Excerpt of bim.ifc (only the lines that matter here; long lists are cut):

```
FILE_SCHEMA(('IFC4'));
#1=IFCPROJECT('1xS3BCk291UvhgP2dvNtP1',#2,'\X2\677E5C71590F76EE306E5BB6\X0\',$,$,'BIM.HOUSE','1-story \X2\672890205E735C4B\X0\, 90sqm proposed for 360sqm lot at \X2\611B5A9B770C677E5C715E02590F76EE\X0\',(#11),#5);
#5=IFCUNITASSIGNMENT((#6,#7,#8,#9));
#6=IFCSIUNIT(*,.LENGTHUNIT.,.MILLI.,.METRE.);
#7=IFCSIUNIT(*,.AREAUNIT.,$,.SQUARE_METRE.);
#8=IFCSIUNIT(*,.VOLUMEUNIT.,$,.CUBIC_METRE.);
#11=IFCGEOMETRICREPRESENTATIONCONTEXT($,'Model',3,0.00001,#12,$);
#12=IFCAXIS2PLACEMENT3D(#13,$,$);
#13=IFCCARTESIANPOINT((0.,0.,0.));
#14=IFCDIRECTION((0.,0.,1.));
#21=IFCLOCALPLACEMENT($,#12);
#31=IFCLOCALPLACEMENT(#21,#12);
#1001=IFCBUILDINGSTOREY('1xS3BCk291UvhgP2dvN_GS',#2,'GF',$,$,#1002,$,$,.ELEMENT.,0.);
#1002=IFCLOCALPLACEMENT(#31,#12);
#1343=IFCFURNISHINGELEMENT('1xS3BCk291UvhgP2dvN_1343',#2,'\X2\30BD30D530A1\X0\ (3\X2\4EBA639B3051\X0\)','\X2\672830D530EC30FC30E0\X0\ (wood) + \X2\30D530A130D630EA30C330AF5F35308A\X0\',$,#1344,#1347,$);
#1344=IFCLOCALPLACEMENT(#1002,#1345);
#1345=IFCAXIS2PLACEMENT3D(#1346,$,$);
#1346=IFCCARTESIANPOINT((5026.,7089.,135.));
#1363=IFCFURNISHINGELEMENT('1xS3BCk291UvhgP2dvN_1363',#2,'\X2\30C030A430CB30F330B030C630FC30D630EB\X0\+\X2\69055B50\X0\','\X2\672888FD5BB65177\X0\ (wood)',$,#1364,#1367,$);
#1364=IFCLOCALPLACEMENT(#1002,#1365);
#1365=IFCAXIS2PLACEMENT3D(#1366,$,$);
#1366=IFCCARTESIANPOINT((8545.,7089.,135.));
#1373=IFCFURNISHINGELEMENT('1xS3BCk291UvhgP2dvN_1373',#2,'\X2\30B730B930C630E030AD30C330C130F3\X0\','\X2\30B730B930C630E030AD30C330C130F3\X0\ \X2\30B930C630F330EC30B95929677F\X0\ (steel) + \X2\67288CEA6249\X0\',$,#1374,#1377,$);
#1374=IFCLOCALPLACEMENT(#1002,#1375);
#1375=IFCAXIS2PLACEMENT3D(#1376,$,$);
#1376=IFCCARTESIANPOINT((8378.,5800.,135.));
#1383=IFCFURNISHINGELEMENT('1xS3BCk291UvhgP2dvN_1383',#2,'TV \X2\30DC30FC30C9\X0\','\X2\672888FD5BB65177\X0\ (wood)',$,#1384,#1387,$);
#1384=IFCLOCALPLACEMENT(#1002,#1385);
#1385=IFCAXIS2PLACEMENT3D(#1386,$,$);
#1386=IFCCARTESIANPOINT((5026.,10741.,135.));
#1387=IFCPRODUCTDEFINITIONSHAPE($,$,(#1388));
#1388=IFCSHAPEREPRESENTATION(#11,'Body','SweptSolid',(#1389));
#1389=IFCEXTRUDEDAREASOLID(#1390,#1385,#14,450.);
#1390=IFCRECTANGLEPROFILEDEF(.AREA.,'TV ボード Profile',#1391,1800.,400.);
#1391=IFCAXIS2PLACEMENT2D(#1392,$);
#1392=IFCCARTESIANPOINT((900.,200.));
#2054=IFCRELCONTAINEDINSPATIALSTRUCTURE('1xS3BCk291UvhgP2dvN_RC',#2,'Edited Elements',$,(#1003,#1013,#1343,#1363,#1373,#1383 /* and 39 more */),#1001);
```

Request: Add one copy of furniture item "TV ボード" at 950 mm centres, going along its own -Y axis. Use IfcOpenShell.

```python
import ifcopenshell
import ifcopenshell.api.geometry
import ifcopenshell.api.root
import ifcopenshell.util.element
import ifcopenshell.util.placement
import ifcopenshell.util.unit

model = ifcopenshell.open("bim.ifc")
unit_scale = ifcopenshell.util.unit.calculate_unit_scale(model)


def reuse_history(source, copy):
    """copy_class also copies each property set's owner history, people and application; keep the originals."""
    for rel in copy.IsDefinedBy:
        if rel.is_a("IfcRelDefinesByProperties") and (history := rel.RelatingPropertyDefinition.OwnerHistory):
            rel.RelatingPropertyDefinition.OwnerHistory = source.OwnerHistory
            ifcopenshell.util.element.remove_deep2(model, history)


source = model.by_guid("1xS3BCk291UvhgP2dvN_1383")
base = ifcopenshell.util.placement.get_local_placement(source.ObjectPlacement)
step = -base[:3, 1] * 0.95 / unit_scale

for i in range(1, 2):
    copy = ifcopenshell.api.root.copy_class(model, product=source)
    copy.Representation = ifcopenshell.util.element.copy_deep(
        model, source.Representation, exclude=["IfcGeometricRepresentationContext", "IfcRepresentationMap"]
    )
    reuse_history(source, copy)
    matrix = base.copy()
    matrix[:3, 3] += i * step
    print("added at", matrix[:3, 3].round(3) + 0.0)
    ifcopenshell.api.geometry.edit_object_placement(model, product=copy, matrix=matrix, is_si=False)

model.write("bim-out.ifc")
```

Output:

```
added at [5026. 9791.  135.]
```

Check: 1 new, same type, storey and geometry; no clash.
